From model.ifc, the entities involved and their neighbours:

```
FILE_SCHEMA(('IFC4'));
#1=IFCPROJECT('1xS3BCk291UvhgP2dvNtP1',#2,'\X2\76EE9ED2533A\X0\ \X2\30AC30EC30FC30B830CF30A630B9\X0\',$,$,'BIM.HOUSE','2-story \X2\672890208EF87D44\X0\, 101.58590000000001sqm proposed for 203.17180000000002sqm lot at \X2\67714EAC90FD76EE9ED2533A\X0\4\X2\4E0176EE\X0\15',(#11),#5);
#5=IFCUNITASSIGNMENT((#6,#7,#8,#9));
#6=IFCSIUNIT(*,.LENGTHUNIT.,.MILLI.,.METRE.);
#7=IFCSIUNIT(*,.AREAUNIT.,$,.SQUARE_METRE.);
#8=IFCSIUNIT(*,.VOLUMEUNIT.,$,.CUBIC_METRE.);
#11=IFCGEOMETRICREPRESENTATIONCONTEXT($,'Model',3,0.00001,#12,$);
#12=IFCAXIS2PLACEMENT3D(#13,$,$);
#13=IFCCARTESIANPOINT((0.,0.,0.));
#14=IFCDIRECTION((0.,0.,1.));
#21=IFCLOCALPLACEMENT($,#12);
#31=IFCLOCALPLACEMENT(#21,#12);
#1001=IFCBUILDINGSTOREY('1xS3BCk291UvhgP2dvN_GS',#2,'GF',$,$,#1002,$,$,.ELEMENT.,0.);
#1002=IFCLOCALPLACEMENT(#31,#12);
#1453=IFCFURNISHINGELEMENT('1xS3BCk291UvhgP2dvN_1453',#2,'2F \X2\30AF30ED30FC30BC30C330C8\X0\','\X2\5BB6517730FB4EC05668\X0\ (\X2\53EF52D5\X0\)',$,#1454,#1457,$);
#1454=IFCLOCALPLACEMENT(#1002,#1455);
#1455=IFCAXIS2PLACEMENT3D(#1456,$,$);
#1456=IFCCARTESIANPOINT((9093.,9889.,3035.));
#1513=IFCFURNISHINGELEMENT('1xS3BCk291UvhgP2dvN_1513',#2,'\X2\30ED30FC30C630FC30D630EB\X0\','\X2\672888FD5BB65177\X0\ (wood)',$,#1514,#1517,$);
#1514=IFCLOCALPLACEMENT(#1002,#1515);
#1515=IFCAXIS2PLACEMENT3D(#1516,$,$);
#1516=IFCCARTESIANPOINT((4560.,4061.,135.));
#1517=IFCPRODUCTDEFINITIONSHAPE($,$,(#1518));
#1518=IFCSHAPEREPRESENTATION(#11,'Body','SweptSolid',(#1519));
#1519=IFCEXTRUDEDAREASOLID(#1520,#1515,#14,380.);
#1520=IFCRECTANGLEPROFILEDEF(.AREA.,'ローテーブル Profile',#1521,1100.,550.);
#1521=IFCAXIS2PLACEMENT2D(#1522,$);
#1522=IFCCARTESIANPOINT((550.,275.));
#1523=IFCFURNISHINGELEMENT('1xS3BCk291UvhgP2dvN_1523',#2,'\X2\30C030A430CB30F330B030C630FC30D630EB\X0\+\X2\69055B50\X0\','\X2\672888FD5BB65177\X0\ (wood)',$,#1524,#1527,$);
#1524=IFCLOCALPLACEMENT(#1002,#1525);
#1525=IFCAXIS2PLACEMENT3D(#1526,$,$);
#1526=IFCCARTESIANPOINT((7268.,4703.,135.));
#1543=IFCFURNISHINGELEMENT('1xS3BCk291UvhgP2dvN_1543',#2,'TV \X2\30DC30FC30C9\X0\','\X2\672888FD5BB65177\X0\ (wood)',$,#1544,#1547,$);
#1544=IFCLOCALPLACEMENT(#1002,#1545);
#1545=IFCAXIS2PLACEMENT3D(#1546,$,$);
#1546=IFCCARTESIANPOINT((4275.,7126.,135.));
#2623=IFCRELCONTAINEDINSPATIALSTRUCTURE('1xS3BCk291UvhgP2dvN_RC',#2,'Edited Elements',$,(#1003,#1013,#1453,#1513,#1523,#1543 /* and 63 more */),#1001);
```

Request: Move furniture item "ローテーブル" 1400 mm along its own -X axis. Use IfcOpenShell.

```python
import ifcopenshell
import ifcopenshell.api.geometry
import ifcopenshell.util.placement

model = ifcopenshell.open("model.ifc")

item = model.by_guid("1xS3BCk291UvhgP2dvN_1513")
matrix = ifcopenshell.util.placement.get_local_placement(item.ObjectPlacement)
matrix[:3, 3] -= matrix[:3, 0] * 1400.0
ifcopenshell.api.geometry.edit_object_placement(model, product=item, matrix=matrix, is_si=False)

print(ifcopenshell.util.placement.get_local_placement(item.ObjectPlacement).round(3) + 0.0)

model.write("model-out.ifc")
```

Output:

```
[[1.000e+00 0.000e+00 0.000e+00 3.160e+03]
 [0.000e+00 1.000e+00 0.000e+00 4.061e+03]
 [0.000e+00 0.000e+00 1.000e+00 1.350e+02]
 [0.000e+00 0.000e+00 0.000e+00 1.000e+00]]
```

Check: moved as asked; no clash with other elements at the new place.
